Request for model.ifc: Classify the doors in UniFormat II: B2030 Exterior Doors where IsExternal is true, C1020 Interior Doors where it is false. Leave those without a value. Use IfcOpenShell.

First a look at what the model holds.

```python
import ifcopenshell
import ifcopenshell.util.element

model = ifcopenshell.open("model.ifc")
print(model.schema)
print("classifications:", [c.Name for c in model.by_type("IfcClassification")])
values = [ifcopenshell.util.element.get_pset(e, "Pset_DoorCommon", "IsExternal") for e in model.by_type("IfcDoor")]
for value in (True, False, None):
    print("IsExternal", value, values.count(value))
```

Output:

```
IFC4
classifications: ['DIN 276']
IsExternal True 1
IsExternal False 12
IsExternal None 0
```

```python
import ifcopenshell
import ifcopenshell.api.classification
import ifcopenshell.util.element

model = ifcopenshell.open("model.ifc")

system = ifcopenshell.api.classification.add_classification(model, classification="UniFormat II")

doors = model.by_type("IfcDoor")
external = {e: ifcopenshell.util.element.get_pset(e, "Pset_DoorCommon", "IsExternal") for e in doors}
for flag, code, name in ((True, "B2030", "Exterior Doors"), (False, "C1020", "Interior Doors")):
    products = [e for e in doors if external[e] is flag]
    ifcopenshell.api.classification.add_reference(
        model, products=products, classification=system, identification=code, name=name
    )
    print(code, len(products))

model.write("model_edited.ifc")
```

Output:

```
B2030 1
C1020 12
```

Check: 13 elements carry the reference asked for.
